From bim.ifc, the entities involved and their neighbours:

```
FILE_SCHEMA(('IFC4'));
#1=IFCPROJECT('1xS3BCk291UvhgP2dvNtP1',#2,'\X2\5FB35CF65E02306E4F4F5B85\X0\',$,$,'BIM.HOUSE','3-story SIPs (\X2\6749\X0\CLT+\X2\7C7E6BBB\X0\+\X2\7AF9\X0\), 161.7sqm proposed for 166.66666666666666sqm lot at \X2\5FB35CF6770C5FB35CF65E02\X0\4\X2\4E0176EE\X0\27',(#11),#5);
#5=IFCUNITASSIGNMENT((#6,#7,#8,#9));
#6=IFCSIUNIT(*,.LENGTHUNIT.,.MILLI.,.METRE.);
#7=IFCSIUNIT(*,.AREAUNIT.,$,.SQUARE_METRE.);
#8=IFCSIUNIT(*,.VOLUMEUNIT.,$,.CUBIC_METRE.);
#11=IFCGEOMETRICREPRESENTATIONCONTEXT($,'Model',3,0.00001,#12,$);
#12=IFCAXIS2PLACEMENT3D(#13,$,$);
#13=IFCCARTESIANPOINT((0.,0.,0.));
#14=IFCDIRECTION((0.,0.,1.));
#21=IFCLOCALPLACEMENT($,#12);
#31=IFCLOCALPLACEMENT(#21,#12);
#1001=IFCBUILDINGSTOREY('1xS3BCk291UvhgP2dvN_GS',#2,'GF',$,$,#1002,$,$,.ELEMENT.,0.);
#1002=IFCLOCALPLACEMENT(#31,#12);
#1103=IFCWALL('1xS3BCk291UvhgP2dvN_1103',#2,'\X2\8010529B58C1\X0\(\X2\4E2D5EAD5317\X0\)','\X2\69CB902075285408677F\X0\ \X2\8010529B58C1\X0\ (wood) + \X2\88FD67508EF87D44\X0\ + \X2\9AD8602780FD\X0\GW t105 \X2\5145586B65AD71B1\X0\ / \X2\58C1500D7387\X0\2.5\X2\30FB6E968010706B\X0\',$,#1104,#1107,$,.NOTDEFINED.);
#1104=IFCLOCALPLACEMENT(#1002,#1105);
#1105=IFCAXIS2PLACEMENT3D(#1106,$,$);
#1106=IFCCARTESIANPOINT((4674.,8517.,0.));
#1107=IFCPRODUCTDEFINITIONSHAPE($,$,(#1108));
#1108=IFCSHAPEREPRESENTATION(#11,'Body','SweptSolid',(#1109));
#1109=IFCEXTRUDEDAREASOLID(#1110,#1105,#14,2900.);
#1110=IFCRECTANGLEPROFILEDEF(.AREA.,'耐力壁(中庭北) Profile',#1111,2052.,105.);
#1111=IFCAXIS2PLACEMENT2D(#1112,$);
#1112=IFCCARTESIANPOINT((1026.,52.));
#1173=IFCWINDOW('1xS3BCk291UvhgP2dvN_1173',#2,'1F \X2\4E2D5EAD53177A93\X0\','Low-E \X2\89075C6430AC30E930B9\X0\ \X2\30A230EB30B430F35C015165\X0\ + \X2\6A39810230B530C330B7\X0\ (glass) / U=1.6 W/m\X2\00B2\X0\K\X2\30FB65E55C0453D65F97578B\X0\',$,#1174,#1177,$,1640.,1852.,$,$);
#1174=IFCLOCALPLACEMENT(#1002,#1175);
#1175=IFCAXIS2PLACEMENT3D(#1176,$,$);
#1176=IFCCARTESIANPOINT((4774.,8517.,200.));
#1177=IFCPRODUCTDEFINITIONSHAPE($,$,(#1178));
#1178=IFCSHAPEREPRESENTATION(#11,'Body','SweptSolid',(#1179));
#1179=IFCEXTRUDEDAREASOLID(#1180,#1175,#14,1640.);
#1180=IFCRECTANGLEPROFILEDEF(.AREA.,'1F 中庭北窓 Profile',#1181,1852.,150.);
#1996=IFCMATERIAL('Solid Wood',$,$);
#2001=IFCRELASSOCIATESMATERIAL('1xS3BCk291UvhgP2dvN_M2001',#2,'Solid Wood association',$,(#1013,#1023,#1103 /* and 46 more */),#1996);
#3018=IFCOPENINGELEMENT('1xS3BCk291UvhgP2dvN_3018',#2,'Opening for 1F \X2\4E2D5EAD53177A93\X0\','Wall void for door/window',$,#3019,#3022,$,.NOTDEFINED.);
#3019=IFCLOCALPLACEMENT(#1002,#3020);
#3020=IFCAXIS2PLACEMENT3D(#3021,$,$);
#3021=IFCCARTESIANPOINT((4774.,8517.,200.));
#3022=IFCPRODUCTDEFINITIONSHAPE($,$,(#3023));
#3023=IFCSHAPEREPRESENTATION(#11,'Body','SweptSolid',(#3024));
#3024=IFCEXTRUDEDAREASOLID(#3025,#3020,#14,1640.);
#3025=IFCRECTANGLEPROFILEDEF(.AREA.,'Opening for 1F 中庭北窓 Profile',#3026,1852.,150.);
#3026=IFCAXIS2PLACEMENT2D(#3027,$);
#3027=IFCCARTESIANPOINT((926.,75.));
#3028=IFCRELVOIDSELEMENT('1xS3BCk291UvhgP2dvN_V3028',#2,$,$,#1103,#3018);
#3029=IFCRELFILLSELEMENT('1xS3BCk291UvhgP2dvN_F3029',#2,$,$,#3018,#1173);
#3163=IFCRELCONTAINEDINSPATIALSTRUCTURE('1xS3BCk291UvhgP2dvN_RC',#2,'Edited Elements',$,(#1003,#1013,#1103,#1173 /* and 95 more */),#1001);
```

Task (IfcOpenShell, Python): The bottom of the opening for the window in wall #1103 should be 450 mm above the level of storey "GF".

```python
import numpy as np
import ifcopenshell
import ifcopenshell.api.geometry
import ifcopenshell.geom
import ifcopenshell.util.element
import ifcopenshell.util.placement
import ifcopenshell.util.shape
import ifcopenshell.util.unit

model = ifcopenshell.open("bim.ifc")
unit_scale = ifcopenshell.util.unit.calculate_unit_scale(model)

window = model.by_id(1173)
opening = window.FillsVoids[0].RelatingOpeningElement
storey = ifcopenshell.util.element.get_container(window, ifc_class="IfcBuildingStorey")
level = ifcopenshell.util.placement.get_local_placement(storey.ObjectPlacement)[2, 3]

# The opening's origin need not be at the sill, so measure its lowest point.
shape = ifcopenshell.geom.create_shape(ifcopenshell.geom.settings(), opening)
bottom = ifcopenshell.util.shape.get_shape_bottom_elevation(shape, shape.geometry) / unit_scale
dz = level + 0.45 / unit_scale - bottom

shift = np.array([0.0, 0.0, dz])
# The window is not placed relative to its opening, so move both.
for product in (opening, window):
    matrix = ifcopenshell.util.placement.get_local_placement(product.ObjectPlacement)
    matrix[:3, 3] += shift
    ifcopenshell.api.geometry.edit_object_placement(model, product=product, matrix=matrix, is_si=False)

print(f"moved by {dz * unit_scale:+.3f} m")

model.write("bim_rev.ifc")
```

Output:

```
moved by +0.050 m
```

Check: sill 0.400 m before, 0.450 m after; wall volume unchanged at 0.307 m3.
